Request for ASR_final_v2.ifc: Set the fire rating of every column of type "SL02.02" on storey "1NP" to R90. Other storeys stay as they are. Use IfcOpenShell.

First a look at what the model holds.

```python
import ifcopenshell
import ifcopenshell.util.element

model = ifcopenshell.open("ASR_final_v2.ifc")
print(model.schema)
storey = next(s for s in model.by_type("IfcBuildingStorey") if s.Name == "1NP")
columns = [e for e in ifcopenshell.util.element.get_decomposition(storey) if e.is_a("IfcColumn")]
seen = {}
for e in columns:
    element_type = ifcopenshell.util.element.get_type(e)
    key = (element_type.Name if element_type != e and element_type else None, ifcopenshell.util.element.get_pset(e, "Pset_ColumnCommon", "FireRating"))
    seen[key] = seen.get(key, 0) + 1
for (name, value), count in sorted(seen.items(), key=str):
    print(count, "x", name, "|", value)
```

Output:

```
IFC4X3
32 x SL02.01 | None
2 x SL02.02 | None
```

```python
import ifcopenshell
import ifcopenshell.api.pset
import ifcopenshell.util.element

model = ifcopenshell.open("ASR_final_v2.ifc")

storey = next(s for s in model.by_type("IfcBuildingStorey") if s.Name == "1NP")
columns = [e for e in ifcopenshell.util.element.get_decomposition(storey) if e.is_a("IfcColumn")]

count = 0
for e in columns:
    element_type = ifcopenshell.util.element.get_type(e)
    if element_type in (None, e) or element_type.Name != "SL02.02":
        continue
    # add_pset returns the element's existing set when there is one.
    pset = ifcopenshell.api.pset.add_pset(model, product=e, name="Pset_ColumnCommon")
    ifcopenshell.api.pset.edit_pset(model, pset=pset, properties={"FireRating": "R90"})
    count += 1

print(count, "columns updated")

model.write("ASR_final_v2_edited.ifc")
```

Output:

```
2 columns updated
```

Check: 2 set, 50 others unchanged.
